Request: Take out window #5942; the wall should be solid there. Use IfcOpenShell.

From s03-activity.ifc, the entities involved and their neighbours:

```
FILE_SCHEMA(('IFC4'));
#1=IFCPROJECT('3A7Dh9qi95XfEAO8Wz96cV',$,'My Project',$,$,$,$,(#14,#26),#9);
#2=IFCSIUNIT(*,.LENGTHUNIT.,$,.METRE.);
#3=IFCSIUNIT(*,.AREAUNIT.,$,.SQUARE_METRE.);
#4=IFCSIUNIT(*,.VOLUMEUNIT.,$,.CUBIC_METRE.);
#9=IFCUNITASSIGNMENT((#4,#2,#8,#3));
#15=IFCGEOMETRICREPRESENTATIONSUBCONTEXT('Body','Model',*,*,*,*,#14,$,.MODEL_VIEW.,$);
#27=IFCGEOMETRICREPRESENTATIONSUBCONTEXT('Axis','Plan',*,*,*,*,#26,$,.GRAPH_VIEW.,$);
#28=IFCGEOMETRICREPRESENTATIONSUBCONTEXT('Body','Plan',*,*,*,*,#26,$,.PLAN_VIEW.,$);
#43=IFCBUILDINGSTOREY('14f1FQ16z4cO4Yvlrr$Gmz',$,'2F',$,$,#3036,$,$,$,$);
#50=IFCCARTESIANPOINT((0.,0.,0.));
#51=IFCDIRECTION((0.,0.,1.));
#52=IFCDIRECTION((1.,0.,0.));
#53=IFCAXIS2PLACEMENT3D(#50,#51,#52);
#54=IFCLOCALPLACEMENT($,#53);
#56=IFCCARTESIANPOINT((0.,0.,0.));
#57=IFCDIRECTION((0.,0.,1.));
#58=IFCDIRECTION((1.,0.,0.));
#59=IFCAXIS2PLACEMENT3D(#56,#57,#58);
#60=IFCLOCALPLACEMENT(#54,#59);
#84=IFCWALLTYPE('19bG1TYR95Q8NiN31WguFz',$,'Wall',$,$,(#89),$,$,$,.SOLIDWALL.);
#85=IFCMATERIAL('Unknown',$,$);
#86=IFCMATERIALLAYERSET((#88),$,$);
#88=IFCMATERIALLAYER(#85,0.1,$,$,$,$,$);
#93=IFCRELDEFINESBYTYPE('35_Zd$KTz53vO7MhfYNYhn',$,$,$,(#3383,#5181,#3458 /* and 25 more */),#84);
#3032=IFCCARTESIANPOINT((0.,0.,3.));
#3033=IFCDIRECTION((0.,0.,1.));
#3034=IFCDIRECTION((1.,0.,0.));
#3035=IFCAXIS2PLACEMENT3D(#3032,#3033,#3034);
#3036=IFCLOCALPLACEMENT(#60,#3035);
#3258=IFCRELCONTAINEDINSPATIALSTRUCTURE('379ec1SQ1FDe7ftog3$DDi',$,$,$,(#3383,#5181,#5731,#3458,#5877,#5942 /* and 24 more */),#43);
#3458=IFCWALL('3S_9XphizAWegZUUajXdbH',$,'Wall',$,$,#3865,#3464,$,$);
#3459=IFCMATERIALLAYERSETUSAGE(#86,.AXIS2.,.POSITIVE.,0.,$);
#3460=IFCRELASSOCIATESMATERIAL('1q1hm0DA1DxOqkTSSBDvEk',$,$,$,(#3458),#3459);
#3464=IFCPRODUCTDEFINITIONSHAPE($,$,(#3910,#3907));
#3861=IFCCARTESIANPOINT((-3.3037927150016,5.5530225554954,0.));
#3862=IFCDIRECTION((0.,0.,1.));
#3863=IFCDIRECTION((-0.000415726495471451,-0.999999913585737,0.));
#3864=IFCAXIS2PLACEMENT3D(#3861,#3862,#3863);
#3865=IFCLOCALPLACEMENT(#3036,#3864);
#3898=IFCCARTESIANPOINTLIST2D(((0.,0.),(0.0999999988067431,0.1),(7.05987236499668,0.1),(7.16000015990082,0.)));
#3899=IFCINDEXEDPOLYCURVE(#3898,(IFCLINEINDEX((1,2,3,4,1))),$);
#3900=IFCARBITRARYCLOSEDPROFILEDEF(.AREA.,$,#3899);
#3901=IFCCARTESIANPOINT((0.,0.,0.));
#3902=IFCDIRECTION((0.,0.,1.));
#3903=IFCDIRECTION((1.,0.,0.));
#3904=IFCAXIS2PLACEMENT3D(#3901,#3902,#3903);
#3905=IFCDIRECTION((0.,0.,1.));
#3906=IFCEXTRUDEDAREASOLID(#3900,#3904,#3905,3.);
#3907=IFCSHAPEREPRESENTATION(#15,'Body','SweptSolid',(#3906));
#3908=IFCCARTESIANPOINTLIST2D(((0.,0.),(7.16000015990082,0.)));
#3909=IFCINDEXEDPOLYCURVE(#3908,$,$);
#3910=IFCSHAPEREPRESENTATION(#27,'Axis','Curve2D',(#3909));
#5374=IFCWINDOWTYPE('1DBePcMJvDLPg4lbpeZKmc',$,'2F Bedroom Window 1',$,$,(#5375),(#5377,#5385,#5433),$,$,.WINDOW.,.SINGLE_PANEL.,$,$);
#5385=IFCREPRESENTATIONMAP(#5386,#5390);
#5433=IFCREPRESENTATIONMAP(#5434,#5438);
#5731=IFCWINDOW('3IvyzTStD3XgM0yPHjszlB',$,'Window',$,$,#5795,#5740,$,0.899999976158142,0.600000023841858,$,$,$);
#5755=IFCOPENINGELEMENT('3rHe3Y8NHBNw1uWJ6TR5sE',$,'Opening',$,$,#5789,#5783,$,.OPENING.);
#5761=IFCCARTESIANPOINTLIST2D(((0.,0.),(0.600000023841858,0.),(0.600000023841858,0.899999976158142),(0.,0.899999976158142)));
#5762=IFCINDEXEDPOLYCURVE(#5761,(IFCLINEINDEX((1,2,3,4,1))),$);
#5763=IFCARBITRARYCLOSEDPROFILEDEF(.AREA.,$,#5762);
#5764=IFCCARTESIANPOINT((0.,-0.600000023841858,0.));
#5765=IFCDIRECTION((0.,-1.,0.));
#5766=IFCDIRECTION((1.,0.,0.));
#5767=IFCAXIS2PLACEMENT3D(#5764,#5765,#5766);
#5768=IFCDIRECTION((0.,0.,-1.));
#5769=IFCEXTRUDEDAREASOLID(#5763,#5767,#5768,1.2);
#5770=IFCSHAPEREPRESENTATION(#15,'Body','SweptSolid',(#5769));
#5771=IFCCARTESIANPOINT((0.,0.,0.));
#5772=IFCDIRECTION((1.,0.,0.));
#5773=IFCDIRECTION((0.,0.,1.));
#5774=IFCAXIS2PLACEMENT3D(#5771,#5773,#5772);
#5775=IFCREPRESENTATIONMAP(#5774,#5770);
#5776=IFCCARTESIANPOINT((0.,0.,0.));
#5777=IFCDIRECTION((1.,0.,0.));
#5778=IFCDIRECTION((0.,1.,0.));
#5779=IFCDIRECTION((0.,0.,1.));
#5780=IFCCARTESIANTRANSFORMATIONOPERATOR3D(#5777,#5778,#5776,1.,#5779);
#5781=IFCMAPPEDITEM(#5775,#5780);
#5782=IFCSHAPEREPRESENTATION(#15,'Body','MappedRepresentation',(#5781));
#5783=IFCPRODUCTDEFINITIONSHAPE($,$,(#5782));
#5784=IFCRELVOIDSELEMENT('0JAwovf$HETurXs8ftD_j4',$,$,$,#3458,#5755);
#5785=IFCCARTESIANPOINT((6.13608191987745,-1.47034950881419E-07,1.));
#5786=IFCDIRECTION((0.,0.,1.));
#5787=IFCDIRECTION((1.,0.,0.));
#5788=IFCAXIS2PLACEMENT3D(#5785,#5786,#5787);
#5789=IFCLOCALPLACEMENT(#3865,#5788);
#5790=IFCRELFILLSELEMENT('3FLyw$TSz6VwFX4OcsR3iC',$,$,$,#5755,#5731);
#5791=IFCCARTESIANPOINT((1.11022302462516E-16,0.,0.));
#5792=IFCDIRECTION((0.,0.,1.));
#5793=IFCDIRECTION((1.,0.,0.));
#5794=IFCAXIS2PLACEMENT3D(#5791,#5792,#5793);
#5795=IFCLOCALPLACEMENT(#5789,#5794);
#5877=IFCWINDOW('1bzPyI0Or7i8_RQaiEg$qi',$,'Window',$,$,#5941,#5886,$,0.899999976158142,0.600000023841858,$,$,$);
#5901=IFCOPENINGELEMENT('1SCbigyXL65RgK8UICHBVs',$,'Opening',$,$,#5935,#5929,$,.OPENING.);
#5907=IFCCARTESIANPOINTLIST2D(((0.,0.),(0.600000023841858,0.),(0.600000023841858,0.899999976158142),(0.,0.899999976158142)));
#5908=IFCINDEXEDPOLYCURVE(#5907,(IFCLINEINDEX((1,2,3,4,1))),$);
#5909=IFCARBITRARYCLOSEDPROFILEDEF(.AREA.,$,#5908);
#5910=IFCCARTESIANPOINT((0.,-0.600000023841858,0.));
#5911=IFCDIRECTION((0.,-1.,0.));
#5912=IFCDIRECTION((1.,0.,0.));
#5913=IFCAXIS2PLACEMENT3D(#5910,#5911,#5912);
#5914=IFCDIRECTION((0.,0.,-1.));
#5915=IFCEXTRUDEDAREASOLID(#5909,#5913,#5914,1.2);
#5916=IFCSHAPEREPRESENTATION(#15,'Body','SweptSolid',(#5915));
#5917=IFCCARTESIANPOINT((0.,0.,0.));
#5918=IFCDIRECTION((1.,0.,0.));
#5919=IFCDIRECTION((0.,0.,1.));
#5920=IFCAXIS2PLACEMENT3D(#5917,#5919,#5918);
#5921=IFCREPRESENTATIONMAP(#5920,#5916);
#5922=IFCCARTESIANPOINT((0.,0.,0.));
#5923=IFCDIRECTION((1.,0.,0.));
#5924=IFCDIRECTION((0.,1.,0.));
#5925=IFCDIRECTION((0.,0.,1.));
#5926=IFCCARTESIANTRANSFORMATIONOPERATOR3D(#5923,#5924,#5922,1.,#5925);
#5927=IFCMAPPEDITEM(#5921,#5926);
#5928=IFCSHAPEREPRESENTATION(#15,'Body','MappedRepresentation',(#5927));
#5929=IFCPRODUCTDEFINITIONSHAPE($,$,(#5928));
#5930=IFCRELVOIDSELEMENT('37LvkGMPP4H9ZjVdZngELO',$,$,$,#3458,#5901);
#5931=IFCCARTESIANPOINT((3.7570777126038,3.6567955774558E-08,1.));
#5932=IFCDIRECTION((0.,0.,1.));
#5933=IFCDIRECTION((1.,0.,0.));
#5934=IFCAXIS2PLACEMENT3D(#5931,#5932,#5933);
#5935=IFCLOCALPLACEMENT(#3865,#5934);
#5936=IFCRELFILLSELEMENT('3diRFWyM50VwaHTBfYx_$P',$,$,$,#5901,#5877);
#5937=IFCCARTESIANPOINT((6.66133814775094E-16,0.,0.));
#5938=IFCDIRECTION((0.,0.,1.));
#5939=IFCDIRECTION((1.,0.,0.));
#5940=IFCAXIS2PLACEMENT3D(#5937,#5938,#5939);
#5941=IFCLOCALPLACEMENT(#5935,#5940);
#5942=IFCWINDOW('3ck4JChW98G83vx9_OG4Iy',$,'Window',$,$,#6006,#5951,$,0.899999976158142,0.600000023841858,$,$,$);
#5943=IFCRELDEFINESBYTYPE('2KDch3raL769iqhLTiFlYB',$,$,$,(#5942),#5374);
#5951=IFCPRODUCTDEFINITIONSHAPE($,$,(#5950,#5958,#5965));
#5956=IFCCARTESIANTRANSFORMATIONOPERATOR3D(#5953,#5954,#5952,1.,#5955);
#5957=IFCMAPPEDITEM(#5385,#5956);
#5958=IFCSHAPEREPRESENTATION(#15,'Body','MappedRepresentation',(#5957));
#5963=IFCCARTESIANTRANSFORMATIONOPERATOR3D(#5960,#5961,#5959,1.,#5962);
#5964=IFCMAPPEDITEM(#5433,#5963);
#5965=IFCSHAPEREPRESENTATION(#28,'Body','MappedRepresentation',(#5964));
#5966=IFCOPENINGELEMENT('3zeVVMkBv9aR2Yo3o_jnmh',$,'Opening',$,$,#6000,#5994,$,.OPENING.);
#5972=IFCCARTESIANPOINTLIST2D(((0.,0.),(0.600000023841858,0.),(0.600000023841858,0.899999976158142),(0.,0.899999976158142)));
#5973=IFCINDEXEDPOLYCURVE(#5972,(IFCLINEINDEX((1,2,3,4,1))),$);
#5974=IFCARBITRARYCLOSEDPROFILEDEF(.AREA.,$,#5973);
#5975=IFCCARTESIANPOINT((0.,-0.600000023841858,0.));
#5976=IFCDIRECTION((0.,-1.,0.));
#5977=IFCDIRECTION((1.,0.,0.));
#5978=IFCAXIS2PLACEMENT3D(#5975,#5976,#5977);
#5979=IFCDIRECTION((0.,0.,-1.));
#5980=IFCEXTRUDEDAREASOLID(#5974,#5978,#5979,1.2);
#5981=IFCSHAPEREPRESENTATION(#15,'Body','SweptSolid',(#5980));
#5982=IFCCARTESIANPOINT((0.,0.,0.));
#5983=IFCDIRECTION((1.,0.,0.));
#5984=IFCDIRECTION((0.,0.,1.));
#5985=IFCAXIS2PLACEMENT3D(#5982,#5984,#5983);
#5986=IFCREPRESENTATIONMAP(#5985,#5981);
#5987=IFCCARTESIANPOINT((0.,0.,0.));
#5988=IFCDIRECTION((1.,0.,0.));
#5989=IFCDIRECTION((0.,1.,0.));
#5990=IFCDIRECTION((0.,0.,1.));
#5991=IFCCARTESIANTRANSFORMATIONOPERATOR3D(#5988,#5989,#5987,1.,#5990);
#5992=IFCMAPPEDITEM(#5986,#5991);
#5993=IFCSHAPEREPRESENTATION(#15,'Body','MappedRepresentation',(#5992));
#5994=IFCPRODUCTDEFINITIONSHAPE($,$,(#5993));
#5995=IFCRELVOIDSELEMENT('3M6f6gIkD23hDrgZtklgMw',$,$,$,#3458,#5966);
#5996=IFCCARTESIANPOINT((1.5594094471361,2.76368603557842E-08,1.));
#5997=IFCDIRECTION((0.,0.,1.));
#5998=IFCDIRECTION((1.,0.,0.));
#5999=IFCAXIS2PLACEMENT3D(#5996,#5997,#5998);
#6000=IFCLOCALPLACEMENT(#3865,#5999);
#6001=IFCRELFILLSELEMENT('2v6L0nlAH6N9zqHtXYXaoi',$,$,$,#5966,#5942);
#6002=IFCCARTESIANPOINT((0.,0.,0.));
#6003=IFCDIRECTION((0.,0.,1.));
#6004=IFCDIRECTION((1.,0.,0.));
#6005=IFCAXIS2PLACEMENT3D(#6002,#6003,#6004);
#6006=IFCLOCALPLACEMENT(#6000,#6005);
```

```python
import ifcopenshell
import ifcopenshell.api.feature
import ifcopenshell.api.root
import ifcopenshell.geom
import ifcopenshell.util.shape

model = ifcopenshell.open("s03-activity.ifc")
settings = ifcopenshell.geom.settings()


def volume(element):
    """Net volume in cubic metres, openings subtracted."""
    shape = ifcopenshell.geom.create_shape(settings, element)
    return ifcopenshell.util.shape.get_volume(shape.geometry)


window = model.by_guid("3ck4JChW98G83vx9_OG4Iy")
opening = window.FillsVoids[0].RelatingOpeningElement
wall = opening.VoidsElements[0].RelatingBuildingElement
before = volume(wall)

ifcopenshell.api.root.remove_product(model, product=window)
ifcopenshell.api.feature.remove_feature(model, feature=opening)

after = volume(wall)

print(f"wall volume {before:.3f} -> {after:.3f} m3")

model.write("s03-activity_v2.ifc")
```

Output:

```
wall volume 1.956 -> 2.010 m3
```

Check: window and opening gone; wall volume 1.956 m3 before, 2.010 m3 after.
